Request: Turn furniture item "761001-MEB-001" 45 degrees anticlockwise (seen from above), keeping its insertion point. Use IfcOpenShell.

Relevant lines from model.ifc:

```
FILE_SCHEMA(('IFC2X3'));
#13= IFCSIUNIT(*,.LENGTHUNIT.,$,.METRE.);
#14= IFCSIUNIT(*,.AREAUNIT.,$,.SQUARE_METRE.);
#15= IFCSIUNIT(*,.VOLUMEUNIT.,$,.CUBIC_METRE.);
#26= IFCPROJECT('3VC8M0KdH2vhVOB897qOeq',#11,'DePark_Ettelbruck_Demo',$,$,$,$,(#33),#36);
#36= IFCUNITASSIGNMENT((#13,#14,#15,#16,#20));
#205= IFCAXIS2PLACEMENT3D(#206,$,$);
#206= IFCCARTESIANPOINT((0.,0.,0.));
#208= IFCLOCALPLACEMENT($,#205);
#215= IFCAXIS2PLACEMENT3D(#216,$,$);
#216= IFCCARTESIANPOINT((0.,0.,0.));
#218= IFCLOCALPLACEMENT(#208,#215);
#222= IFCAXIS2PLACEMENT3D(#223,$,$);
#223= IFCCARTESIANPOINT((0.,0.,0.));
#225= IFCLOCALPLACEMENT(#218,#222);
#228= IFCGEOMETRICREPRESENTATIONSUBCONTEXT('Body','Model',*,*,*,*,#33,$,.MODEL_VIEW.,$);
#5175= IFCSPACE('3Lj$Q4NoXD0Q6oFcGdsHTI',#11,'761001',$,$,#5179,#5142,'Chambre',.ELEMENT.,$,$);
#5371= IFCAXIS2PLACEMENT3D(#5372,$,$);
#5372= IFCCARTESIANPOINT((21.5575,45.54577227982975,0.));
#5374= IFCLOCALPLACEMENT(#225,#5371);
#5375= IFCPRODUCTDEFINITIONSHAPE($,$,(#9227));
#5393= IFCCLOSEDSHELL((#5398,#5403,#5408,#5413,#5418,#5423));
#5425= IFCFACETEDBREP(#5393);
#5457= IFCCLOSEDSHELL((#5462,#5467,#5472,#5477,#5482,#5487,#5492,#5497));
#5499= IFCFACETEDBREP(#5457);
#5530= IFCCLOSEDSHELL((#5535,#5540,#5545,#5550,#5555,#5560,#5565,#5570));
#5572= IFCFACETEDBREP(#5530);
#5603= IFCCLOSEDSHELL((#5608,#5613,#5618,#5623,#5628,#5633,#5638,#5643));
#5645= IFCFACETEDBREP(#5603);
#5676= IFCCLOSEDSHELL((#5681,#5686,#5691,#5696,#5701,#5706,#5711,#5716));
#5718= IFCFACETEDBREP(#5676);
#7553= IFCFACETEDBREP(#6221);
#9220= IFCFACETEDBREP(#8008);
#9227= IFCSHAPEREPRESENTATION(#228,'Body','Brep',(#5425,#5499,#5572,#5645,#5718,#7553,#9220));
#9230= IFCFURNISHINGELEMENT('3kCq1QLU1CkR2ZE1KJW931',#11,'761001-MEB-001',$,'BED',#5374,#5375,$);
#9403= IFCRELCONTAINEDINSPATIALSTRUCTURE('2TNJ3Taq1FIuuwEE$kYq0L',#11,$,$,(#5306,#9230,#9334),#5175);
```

```python
import ifcopenshell
import ifcopenshell.api.geometry
import ifcopenshell.util.placement

model = ifcopenshell.open("model.ifc")

item = model.by_id(9230)
matrix = ifcopenshell.util.placement.get_local_placement(item.ObjectPlacement)
matrix = matrix @ ifcopenshell.util.placement.rotation(45, "Z")
ifcopenshell.api.geometry.edit_object_placement(model, product=item, matrix=matrix, is_si=False)

print(ifcopenshell.util.placement.get_local_placement(item.ObjectPlacement).round(3) + 0.0)

model.write("model_edited.ifc")
```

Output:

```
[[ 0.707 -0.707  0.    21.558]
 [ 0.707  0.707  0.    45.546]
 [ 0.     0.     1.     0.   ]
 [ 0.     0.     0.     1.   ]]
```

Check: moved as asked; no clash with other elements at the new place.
